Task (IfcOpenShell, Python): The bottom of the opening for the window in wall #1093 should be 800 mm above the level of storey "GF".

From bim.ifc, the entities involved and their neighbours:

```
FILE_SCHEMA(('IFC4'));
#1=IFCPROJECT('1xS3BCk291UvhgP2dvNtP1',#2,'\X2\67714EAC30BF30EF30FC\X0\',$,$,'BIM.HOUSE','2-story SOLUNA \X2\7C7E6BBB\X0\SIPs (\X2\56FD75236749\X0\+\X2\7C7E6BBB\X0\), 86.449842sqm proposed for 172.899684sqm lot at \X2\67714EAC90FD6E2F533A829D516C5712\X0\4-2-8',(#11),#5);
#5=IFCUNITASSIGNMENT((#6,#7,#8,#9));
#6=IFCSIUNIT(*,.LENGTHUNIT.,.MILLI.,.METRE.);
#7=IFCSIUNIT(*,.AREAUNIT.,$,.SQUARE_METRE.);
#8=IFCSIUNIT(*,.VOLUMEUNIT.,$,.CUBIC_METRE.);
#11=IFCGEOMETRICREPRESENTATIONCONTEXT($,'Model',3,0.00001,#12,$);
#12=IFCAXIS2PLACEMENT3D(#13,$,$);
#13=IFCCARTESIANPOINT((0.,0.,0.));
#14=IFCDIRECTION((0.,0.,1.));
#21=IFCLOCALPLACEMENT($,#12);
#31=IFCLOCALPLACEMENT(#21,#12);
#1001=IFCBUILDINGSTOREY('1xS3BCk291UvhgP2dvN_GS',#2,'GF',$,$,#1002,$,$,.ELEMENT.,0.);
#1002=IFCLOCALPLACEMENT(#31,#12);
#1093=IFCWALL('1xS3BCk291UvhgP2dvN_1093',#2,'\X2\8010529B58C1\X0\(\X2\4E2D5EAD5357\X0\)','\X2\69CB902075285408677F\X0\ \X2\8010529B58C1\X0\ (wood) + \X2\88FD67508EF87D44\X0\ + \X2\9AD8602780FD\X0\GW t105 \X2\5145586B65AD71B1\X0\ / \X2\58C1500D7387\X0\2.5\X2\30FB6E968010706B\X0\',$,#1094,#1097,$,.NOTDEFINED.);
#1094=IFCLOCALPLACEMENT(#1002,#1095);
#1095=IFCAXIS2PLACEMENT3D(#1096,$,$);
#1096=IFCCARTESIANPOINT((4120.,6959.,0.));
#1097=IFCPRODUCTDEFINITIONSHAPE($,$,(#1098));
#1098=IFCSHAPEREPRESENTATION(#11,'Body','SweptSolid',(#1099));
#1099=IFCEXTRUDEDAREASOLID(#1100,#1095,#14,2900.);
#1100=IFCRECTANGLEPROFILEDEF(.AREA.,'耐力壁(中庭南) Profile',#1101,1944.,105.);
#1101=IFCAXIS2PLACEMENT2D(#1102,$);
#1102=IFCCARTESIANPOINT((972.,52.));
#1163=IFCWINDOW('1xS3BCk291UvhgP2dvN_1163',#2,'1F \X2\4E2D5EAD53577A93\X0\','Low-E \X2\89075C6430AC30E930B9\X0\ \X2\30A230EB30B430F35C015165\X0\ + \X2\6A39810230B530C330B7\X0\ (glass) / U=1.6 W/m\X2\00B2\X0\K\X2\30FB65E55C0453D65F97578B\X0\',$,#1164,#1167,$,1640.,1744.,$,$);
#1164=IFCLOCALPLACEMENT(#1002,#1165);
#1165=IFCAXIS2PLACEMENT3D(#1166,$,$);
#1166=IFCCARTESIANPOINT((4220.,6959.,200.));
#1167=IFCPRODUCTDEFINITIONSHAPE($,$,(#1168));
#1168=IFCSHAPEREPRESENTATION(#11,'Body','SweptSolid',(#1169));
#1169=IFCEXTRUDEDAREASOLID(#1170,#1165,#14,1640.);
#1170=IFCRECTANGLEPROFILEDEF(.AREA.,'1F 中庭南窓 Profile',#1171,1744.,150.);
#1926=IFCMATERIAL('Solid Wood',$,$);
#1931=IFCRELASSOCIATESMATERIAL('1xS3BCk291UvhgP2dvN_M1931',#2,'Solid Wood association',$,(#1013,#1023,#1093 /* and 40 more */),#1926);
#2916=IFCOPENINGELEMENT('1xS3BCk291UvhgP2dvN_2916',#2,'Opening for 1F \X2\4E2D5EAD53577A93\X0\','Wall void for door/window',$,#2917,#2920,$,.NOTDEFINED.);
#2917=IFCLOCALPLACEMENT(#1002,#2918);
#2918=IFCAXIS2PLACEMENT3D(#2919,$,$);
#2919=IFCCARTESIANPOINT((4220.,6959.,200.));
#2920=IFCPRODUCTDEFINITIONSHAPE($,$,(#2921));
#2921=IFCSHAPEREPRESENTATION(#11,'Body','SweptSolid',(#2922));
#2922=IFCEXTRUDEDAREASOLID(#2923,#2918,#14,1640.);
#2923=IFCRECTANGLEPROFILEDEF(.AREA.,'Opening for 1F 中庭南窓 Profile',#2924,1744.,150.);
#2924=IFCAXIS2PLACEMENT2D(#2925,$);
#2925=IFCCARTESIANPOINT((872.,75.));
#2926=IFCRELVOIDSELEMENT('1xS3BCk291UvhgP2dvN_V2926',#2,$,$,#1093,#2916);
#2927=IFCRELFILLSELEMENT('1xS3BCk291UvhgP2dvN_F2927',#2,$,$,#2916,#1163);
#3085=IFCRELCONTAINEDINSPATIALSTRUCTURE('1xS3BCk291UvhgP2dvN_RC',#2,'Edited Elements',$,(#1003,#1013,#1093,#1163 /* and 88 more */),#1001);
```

```python
import numpy as np
import ifcopenshell
import ifcopenshell.api.geometry
import ifcopenshell.geom
import ifcopenshell.util.element
import ifcopenshell.util.placement
import ifcopenshell.util.shape
import ifcopenshell.util.unit

model = ifcopenshell.open("bim.ifc")
unit_scale = ifcopenshell.util.unit.calculate_unit_scale(model)

window = model.by_guid("1xS3BCk291UvhgP2dvN_1163")
opening = window.FillsVoids[0].RelatingOpeningElement
storey = ifcopenshell.util.element.get_container(window, ifc_class="IfcBuildingStorey")
level = ifcopenshell.util.placement.get_local_placement(storey.ObjectPlacement)[2, 3]

# The opening's origin need not be at the sill, so measure its lowest point.
shape = ifcopenshell.geom.create_shape(ifcopenshell.geom.settings(), opening)
bottom = ifcopenshell.util.shape.get_shape_bottom_elevation(shape, shape.geometry) / unit_scale
dz = level + 800.0 - bottom

shift = np.array([0.0, 0.0, dz])
# The window is not placed relative to its opening, so move both.
for product in (opening, window):
    matrix = ifcopenshell.util.placement.get_local_placement(product.ObjectPlacement)
    matrix[:3, 3] += shift
    ifcopenshell.api.geometry.edit_object_placement(model, product=product, matrix=matrix, is_si=False)

print(f"moved by {dz * unit_scale:+.3f} m")

model.write("bim_edited.ifc")
```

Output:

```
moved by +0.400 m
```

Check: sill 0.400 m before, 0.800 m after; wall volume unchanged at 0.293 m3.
